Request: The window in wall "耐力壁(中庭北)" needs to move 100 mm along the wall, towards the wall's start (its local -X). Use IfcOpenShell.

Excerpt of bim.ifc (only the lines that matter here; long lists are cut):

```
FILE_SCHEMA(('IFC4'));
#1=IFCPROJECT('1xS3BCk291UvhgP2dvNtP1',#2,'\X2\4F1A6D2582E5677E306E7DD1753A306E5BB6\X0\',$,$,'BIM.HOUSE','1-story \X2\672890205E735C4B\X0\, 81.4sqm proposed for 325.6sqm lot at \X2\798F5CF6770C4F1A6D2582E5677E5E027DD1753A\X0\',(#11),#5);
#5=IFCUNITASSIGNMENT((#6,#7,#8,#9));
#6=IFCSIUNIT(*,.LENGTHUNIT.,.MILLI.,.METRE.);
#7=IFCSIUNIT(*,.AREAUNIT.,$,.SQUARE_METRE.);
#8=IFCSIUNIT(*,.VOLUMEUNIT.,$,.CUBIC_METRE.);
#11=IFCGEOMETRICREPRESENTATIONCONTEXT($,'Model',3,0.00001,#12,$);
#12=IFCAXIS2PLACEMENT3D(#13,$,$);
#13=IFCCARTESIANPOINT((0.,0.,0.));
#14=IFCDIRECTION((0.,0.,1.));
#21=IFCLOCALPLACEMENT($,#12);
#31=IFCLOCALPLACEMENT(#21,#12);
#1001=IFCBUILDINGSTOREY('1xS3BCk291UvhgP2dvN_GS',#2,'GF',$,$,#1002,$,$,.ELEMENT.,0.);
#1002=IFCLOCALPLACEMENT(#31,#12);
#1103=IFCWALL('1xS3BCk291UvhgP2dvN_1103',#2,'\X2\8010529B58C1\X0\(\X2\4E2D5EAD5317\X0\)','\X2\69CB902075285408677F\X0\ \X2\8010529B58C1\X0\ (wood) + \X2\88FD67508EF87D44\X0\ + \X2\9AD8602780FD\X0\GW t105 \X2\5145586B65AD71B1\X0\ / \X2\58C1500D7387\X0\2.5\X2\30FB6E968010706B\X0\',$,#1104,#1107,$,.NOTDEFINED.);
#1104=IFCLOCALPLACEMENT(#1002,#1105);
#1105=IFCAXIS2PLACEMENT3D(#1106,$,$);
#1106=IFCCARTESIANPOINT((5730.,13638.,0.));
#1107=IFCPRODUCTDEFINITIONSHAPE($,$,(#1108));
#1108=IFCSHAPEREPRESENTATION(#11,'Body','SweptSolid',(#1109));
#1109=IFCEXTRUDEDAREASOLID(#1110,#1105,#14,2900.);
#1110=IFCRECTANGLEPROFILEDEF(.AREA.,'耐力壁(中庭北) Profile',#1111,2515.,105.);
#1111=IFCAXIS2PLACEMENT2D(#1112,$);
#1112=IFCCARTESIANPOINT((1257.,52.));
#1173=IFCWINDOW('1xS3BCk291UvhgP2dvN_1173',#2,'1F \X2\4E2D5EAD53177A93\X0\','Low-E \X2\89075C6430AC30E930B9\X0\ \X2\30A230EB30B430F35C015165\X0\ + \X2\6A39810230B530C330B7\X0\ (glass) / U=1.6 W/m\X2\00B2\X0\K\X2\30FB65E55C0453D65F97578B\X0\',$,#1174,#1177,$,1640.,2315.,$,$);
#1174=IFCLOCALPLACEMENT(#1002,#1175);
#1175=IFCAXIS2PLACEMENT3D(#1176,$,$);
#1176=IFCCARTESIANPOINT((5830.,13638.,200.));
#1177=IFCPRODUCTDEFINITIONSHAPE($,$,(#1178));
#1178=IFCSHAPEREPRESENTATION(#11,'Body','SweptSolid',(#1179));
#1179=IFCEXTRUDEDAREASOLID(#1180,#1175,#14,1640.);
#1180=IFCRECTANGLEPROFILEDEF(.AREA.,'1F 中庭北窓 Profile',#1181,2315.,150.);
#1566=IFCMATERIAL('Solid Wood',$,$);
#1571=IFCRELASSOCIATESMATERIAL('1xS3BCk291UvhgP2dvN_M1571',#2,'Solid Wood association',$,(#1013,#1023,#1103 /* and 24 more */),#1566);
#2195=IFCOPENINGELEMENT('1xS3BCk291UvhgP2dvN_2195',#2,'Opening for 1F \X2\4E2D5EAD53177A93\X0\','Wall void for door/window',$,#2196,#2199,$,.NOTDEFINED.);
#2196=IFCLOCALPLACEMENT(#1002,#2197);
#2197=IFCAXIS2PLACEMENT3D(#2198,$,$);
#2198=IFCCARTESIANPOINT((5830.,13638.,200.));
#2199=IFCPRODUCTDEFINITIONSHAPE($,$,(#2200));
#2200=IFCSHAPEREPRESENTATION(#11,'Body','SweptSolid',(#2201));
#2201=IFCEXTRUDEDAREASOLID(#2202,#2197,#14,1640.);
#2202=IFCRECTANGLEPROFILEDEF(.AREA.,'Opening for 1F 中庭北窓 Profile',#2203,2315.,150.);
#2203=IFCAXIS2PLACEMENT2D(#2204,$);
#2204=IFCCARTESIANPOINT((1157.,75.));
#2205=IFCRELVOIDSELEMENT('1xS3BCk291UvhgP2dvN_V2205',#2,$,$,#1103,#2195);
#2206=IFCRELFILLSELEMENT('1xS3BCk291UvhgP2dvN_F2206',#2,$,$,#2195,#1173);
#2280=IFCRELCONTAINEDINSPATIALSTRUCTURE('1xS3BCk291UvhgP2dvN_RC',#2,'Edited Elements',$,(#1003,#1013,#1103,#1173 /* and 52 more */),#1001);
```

```python
import ifcopenshell
import ifcopenshell.api.geometry
import ifcopenshell.util.placement
import ifcopenshell.util.unit

model = ifcopenshell.open("bim.ifc")
unit_scale = ifcopenshell.util.unit.calculate_unit_scale(model)

window = model.by_id(1173)
opening = window.FillsVoids[0].RelatingOpeningElement
wall = opening.VoidsElements[0].RelatingBuildingElement

wall_matrix = ifcopenshell.util.placement.get_local_placement(wall.ObjectPlacement)
shift = wall_matrix[:3, 0] * -0.1 / unit_scale
before = ifcopenshell.util.placement.get_local_placement(window.ObjectPlacement)[:3, 3].copy()

# The window is not placed relative to its opening, so move both.
for product in (opening, window):
    matrix = ifcopenshell.util.placement.get_local_placement(product.ObjectPlacement)
    matrix[:3, 3] += shift
    ifcopenshell.api.geometry.edit_object_placement(model, product=product, matrix=matrix, is_si=False)

after = ifcopenshell.util.placement.get_local_placement(window.ObjectPlacement)[:3, 3]
print("window moved by", (after - before).round(3) + 0.0)

model.write("bim-out.ifc")
```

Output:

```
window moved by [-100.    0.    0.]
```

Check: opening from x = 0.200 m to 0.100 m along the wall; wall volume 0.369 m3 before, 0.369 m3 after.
